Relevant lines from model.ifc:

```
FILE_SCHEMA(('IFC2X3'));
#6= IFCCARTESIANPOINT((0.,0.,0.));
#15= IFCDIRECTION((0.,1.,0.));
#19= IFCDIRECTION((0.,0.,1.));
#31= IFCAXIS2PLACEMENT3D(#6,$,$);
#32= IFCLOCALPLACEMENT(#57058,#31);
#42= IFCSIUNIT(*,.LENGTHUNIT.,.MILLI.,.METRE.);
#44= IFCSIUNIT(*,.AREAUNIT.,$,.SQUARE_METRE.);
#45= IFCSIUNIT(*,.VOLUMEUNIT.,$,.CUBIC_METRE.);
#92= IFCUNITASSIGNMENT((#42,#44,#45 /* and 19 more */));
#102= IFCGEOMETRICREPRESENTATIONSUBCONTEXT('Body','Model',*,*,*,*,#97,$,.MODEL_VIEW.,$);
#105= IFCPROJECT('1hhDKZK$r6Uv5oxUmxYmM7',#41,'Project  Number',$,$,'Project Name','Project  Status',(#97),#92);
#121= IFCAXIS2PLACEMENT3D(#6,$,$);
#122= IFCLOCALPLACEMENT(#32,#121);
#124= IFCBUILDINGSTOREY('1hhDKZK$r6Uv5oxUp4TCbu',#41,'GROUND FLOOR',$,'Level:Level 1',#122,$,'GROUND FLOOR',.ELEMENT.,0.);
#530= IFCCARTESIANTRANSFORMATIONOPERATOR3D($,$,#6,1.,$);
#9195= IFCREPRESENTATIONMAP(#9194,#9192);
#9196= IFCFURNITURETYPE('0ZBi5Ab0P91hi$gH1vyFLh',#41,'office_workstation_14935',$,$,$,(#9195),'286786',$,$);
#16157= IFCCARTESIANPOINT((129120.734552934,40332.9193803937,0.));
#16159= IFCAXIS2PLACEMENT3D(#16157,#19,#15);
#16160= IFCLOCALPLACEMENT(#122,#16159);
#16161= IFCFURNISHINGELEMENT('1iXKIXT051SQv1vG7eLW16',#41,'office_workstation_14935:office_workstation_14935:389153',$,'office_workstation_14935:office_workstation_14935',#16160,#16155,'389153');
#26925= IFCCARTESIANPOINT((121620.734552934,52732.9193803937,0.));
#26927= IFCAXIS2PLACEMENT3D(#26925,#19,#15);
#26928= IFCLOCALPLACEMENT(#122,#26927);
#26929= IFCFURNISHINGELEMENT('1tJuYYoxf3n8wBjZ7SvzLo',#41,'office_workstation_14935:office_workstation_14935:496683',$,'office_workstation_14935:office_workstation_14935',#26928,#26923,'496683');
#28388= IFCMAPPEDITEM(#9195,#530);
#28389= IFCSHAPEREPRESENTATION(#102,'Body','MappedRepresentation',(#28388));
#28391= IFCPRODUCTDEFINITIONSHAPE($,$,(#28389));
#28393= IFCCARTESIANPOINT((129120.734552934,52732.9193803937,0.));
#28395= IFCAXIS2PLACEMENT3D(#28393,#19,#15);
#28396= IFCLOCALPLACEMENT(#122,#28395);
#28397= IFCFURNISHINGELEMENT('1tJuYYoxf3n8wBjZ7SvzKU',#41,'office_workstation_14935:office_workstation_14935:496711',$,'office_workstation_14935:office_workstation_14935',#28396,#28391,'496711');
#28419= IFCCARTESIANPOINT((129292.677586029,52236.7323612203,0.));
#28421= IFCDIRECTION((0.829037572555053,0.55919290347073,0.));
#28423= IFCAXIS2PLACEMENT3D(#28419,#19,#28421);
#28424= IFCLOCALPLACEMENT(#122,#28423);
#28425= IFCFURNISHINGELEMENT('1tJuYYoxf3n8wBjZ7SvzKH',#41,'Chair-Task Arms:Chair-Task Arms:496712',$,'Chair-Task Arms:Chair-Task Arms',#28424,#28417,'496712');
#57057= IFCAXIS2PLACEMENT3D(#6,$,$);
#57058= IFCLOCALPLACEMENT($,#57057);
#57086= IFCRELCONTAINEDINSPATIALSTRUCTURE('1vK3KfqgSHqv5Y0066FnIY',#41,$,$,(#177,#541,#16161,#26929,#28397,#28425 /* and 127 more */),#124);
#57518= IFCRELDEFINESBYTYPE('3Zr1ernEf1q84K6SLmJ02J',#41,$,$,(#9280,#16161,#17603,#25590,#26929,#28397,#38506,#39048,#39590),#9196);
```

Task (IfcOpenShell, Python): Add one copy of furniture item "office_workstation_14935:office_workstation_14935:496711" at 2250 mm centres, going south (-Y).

```python
import numpy as np
import ifcopenshell
import ifcopenshell.api.geometry
import ifcopenshell.api.root
import ifcopenshell.util.element
import ifcopenshell.util.placement
import ifcopenshell.util.unit

model = ifcopenshell.open("model.ifc")
unit_scale = ifcopenshell.util.unit.calculate_unit_scale(model)


def reuse_history(source, copy):
    """copy_class also copies each property set's owner history, people and application; keep the originals."""
    for rel in copy.IsDefinedBy:
        if rel.is_a("IfcRelDefinesByProperties") and (history := rel.RelatingPropertyDefinition.OwnerHistory):
            rel.RelatingPropertyDefinition.OwnerHistory = source.OwnerHistory
            ifcopenshell.util.element.remove_deep2(model, history)


source = model.by_guid("1tJuYYoxf3n8wBjZ7SvzKU")
base = ifcopenshell.util.placement.get_local_placement(source.ObjectPlacement)
step = np.array([0.0, -1.0, 0.0]) * 2.25 / unit_scale

for i in range(1, 2):
    copy = ifcopenshell.api.root.copy_class(model, product=source)
    copy.Representation = ifcopenshell.util.element.copy_deep(
        model, source.Representation, exclude=["IfcGeometricRepresentationContext", "IfcRepresentationMap"]
    )
    copy.Name = "office_workstation_14935:office_workstation_14935"
    copy.Tag = None
    reuse_history(source, copy)
    matrix = base.copy()
    matrix[:3, 3] += i * step
    print("added at", matrix[:3, 3].round(3) + 0.0)
    ifcopenshell.api.geometry.edit_object_placement(model, product=copy, matrix=matrix, is_si=False)

model.write("model_edited.ifc")
```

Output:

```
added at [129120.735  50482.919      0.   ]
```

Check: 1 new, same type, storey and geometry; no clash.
